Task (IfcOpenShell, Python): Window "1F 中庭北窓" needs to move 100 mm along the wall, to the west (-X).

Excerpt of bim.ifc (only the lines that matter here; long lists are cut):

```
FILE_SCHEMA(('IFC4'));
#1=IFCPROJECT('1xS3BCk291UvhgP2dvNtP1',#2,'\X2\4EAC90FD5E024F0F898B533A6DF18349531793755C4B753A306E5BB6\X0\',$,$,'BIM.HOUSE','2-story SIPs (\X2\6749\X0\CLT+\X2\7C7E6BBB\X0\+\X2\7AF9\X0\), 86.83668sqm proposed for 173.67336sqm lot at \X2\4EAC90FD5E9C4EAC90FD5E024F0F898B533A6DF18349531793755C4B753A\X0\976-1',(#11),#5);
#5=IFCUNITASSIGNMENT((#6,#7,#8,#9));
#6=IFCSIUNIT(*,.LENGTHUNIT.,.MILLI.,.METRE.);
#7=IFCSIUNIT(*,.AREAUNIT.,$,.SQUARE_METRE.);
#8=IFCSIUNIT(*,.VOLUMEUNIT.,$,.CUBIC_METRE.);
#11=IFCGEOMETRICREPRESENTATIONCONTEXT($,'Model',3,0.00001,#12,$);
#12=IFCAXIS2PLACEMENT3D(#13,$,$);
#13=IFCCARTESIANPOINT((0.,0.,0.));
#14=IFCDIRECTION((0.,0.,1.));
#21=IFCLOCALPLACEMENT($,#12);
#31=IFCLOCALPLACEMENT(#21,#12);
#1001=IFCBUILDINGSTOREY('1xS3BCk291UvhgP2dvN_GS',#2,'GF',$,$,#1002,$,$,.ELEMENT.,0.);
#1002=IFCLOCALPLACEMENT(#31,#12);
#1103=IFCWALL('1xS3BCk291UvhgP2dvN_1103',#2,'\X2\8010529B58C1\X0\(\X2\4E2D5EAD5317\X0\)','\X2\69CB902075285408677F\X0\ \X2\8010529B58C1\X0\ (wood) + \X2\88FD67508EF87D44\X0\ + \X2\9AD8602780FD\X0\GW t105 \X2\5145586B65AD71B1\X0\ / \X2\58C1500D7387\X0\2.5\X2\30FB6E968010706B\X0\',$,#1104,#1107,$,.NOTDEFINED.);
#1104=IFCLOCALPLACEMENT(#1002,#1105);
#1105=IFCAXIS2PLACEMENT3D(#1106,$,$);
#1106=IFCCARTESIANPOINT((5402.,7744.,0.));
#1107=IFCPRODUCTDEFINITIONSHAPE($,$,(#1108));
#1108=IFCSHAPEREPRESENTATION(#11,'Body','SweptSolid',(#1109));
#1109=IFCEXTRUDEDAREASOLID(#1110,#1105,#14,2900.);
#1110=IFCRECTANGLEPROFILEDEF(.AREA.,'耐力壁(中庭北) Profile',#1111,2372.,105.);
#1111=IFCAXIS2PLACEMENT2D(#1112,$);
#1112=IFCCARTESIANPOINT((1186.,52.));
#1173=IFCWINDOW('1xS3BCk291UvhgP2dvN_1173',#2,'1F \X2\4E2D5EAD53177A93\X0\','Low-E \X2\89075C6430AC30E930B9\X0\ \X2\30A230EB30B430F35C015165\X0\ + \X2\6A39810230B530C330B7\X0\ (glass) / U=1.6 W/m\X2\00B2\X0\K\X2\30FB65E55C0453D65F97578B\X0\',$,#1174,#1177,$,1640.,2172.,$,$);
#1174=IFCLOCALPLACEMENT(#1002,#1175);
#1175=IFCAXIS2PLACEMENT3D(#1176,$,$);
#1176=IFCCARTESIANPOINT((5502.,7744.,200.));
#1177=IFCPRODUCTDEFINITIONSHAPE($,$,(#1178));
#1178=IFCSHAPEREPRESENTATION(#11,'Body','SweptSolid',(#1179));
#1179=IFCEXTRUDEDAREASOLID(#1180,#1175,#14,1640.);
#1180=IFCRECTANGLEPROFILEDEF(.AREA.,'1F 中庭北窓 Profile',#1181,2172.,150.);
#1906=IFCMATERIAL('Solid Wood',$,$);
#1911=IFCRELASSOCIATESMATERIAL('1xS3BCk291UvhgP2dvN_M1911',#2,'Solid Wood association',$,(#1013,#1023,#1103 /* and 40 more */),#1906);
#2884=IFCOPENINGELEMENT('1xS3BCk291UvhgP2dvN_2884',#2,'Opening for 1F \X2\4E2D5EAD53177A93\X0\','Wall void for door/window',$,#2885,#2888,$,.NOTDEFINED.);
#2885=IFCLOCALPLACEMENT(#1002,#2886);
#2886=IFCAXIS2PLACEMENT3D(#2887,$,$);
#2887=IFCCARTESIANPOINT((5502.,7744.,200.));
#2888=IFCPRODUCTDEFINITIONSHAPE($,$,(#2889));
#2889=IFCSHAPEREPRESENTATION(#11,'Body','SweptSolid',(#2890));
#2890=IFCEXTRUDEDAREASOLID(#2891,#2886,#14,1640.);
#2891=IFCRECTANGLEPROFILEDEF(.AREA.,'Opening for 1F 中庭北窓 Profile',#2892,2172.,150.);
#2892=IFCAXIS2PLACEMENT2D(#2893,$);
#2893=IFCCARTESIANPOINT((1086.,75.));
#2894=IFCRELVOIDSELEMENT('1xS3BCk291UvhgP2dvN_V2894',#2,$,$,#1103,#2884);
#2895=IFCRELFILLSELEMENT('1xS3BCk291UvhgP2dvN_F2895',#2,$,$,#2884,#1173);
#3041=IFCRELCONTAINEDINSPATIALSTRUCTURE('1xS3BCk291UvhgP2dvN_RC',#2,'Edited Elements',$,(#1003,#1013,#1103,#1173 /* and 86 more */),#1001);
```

```python
import ifcopenshell
import ifcopenshell.api.geometry
import ifcopenshell.util.placement
import ifcopenshell.util.unit

model = ifcopenshell.open("bim.ifc")
unit_scale = ifcopenshell.util.unit.calculate_unit_scale(model)

window = model.by_guid("1xS3BCk291UvhgP2dvN_1173")
opening = window.FillsVoids[0].RelatingOpeningElement
wall = opening.VoidsElements[0].RelatingBuildingElement

wall_matrix = ifcopenshell.util.placement.get_local_placement(wall.ObjectPlacement)
shift = wall_matrix[:3, 0] * -0.1 / unit_scale
before = ifcopenshell.util.placement.get_local_placement(window.ObjectPlacement)[:3, 3].copy()

# The window is not placed relative to its opening, so move both.
for product in (opening, window):
    matrix = ifcopenshell.util.placement.get_local_placement(product.ObjectPlacement)
    matrix[:3, 3] += shift
    ifcopenshell.api.geometry.edit_object_placement(model, product=product, matrix=matrix, is_si=False)

after = ifcopenshell.util.placement.get_local_placement(window.ObjectPlacement)[:3, 3]
print("window moved by", (after - before).round(3) + 0.0)

model.write("bim_rev.ifc")
```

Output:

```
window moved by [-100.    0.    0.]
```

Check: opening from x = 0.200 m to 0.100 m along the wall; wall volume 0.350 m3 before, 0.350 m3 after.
